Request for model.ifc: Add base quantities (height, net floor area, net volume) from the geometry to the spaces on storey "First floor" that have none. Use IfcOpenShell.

First a look at what the model holds.

```python
import ifcopenshell
import ifcopenshell.util.element
import ifcopenshell.util.unit

model = ifcopenshell.open("model.ifc")
print(model.schema)
for unit_type in ("LENGTHUNIT", "AREAUNIT", "VOLUMEUNIT"):
    print(unit_type, ifcopenshell.util.unit.calculate_unit_scale(model, unit_type))
storey = next(s for s in model.by_type("IfcBuildingStorey") if s.Name == "First floor")
spaces = [e for e in ifcopenshell.util.element.get_decomposition(storey) if e.is_a("IfcSpace")]
for e in sorted(spaces, key=lambda e: e.id()):
    print(e.id(), e.is_a(), e.Name, list(ifcopenshell.util.element.get_psets(e, qtos_only=True)), sep=" | ")
```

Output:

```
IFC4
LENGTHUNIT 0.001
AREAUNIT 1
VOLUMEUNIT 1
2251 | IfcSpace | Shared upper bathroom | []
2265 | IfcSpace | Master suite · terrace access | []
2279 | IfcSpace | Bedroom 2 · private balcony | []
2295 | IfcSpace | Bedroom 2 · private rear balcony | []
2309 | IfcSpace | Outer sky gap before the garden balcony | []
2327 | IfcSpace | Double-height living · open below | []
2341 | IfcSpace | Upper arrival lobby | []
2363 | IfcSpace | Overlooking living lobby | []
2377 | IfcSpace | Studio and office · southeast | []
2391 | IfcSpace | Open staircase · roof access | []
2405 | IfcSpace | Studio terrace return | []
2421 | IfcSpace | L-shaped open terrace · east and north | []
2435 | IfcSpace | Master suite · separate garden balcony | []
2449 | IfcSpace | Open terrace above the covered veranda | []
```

```python
import ifcopenshell
import ifcopenshell.api.pset
import ifcopenshell.geom
import ifcopenshell.util.element
import ifcopenshell.util.shape
import ifcopenshell.util.unit

model = ifcopenshell.open("model.ifc")
unit_scale = ifcopenshell.util.unit.calculate_unit_scale(model)
area_scale = ifcopenshell.util.unit.calculate_unit_scale(model, "AREAUNIT")
volume_scale = ifcopenshell.util.unit.calculate_unit_scale(model, "VOLUMEUNIT")
settings = ifcopenshell.geom.settings()

storey = next(s for s in model.by_type("IfcBuildingStorey") if s.Name == "First floor")
spaces = [e for e in ifcopenshell.util.element.get_decomposition(storey) if e.is_a("IfcSpace")]

for e in sorted(spaces, key=lambda e: e.id()):
    if ifcopenshell.util.element.get_psets(e, qtos_only=True, should_inherit=False):
        continue
    # Geometry comes back in metres, in the element's own axes.
    shape = ifcopenshell.geom.create_shape(settings, e)
    values = {
        "Height": ifcopenshell.util.shape.get_z(shape.geometry) / unit_scale,
        "NetFloorArea": ifcopenshell.util.shape.get_footprint_area(shape.geometry) / area_scale,
        "NetVolume": ifcopenshell.util.shape.get_volume(shape.geometry) / volume_scale,
    }
    qto = ifcopenshell.api.pset.add_qto(model, product=e, name="Qto_SpaceBaseQuantities")
    ifcopenshell.api.pset.edit_qto(model, qto=qto, properties=values)
    print(e.id(), {k: round(v, 3) for k, v in values.items()})

model.write("model-out.ifc")
```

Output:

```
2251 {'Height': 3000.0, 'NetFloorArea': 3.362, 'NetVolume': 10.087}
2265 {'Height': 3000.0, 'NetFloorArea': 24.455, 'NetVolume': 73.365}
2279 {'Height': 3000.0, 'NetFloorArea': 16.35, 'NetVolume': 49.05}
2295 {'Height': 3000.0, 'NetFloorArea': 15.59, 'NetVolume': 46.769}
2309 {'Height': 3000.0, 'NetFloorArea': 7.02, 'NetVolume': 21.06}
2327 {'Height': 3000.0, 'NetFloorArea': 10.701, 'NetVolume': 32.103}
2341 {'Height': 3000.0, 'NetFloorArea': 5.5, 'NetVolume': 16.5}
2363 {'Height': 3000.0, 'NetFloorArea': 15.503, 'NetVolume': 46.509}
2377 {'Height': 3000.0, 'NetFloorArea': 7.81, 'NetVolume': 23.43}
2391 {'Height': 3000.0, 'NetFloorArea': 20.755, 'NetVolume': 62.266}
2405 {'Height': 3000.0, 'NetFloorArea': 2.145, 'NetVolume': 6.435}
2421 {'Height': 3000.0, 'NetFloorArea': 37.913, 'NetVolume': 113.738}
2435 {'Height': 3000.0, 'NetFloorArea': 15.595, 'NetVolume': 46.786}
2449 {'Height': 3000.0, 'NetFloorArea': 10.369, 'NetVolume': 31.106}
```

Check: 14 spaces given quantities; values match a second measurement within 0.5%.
